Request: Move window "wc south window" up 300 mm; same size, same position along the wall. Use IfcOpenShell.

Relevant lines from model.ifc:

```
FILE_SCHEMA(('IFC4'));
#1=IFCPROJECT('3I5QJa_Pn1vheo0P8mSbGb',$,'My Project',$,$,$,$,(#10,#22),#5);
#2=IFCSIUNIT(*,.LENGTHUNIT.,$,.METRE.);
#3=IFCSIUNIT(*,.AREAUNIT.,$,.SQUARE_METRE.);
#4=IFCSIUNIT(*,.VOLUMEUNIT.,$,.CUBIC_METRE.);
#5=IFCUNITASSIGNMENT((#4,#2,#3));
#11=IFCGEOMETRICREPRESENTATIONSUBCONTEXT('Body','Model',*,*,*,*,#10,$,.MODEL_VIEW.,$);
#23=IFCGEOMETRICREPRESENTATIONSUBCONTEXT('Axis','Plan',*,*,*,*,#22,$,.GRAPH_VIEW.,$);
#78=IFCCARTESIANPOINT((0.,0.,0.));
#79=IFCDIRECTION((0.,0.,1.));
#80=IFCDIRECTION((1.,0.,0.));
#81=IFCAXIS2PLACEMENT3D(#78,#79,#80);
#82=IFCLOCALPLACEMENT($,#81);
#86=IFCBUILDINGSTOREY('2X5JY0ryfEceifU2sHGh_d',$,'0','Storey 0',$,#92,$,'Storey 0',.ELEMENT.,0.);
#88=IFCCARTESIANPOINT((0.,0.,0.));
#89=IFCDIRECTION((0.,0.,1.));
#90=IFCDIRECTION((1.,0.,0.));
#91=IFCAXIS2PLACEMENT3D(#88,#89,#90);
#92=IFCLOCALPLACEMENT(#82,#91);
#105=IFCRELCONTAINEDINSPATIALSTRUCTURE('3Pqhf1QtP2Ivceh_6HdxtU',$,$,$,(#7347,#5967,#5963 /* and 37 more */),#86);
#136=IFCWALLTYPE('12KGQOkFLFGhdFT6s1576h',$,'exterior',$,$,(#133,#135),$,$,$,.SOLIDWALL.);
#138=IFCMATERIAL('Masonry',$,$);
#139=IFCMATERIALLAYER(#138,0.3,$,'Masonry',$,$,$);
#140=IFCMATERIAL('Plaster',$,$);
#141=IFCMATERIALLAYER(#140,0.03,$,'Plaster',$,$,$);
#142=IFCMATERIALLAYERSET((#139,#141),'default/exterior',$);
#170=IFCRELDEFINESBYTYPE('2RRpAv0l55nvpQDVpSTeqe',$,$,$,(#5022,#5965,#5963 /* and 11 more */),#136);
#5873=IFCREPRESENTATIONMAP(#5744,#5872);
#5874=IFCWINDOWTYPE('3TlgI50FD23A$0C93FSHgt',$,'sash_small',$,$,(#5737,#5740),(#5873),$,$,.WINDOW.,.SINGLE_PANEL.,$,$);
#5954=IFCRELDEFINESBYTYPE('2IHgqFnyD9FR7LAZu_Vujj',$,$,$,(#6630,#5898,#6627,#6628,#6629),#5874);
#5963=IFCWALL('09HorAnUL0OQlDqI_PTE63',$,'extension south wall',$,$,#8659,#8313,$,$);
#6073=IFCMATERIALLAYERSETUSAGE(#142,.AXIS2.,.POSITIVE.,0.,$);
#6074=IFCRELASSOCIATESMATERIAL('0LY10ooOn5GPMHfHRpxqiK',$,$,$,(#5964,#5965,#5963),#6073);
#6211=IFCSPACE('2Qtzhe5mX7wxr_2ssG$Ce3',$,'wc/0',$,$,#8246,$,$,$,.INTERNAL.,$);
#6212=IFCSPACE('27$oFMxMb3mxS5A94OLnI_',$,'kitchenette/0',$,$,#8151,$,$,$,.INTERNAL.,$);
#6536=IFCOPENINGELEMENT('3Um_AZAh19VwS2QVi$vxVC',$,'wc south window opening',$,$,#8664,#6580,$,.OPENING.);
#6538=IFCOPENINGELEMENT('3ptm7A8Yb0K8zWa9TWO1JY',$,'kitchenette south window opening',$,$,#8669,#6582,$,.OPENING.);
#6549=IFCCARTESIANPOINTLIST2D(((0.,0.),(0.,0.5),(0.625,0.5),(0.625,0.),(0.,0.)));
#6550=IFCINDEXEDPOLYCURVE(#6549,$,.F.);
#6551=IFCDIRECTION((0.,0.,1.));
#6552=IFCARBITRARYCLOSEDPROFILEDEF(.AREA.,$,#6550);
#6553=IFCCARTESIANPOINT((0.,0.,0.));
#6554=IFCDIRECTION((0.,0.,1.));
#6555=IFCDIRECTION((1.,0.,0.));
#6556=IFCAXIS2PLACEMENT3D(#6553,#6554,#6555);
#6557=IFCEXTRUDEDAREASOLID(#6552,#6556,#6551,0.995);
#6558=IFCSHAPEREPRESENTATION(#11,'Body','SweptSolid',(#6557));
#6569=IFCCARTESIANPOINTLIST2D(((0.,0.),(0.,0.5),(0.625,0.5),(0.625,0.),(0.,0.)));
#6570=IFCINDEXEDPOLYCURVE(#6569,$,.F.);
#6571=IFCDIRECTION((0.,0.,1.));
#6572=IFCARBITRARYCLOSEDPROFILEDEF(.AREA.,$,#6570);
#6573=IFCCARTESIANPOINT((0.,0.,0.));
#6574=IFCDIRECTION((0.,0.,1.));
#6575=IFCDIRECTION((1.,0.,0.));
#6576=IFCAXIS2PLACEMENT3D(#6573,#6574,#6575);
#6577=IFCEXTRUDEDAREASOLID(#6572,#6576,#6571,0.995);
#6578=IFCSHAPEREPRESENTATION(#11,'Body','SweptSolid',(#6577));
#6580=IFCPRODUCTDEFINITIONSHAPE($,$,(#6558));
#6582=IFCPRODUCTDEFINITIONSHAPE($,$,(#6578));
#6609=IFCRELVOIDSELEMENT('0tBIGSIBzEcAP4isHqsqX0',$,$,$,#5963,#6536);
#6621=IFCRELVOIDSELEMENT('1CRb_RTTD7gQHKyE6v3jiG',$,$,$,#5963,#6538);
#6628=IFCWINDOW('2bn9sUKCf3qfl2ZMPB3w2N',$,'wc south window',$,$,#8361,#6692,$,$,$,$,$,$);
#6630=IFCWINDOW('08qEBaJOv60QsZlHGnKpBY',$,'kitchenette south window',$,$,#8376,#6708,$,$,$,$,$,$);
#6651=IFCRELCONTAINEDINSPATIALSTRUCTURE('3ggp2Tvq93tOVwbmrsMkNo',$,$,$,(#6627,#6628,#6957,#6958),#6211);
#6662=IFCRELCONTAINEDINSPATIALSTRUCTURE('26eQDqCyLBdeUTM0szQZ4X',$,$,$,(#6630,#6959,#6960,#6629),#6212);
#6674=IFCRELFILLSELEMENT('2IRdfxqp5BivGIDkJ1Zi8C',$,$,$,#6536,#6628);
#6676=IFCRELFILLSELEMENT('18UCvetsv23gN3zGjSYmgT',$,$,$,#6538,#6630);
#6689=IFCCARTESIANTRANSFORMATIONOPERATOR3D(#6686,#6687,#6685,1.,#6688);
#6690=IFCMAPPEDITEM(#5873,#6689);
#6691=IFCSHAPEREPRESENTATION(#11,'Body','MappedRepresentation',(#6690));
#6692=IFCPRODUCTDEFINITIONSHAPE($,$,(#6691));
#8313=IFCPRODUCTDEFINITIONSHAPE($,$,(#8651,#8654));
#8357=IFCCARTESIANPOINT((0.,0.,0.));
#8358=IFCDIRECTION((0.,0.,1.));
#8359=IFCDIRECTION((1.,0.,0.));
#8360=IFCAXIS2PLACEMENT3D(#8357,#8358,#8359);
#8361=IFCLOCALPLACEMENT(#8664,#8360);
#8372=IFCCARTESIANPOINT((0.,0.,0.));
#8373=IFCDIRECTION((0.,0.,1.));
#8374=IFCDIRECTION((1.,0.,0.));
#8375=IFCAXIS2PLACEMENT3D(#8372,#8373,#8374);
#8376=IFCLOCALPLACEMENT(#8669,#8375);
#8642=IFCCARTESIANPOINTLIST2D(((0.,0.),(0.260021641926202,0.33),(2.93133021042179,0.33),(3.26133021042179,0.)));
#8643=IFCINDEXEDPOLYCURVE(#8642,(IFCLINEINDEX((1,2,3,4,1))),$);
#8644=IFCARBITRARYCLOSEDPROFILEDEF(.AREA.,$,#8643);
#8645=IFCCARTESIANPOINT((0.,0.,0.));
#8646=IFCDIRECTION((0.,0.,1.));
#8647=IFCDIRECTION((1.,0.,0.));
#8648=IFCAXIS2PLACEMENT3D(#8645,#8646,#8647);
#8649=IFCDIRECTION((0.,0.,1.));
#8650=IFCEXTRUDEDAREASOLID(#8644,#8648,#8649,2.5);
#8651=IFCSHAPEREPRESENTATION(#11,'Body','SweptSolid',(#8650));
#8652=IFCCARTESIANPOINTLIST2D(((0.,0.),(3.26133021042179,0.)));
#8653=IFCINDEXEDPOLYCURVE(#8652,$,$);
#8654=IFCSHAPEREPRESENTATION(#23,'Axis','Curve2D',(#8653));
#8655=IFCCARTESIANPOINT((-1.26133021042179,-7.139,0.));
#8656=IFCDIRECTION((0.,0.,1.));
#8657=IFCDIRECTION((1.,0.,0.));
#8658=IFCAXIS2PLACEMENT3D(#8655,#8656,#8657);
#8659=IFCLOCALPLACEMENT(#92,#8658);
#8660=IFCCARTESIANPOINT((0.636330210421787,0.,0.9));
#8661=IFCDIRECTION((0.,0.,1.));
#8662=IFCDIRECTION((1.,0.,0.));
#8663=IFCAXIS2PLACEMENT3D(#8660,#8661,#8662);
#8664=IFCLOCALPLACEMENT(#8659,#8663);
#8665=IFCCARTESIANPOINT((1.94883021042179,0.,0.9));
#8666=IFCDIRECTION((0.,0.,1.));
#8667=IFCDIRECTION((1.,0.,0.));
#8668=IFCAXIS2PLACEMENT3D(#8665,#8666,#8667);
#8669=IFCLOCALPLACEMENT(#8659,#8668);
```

```python
import numpy as np
import ifcopenshell
import ifcopenshell.api.geometry
import ifcopenshell.util.placement
import ifcopenshell.util.unit

model = ifcopenshell.open("model.ifc")
unit_scale = ifcopenshell.util.unit.calculate_unit_scale(model)

window = model.by_id(6628)
opening = window.FillsVoids[0].RelatingOpeningElement
dz = 0.3

shift = np.array([0.0, 0.0, dz])
# The window is placed relative to its opening, so it follows when the opening moves.
matrix = ifcopenshell.util.placement.get_local_placement(opening.ObjectPlacement)
matrix[:3, 3] += shift
ifcopenshell.api.geometry.edit_object_placement(
    model, product=opening, matrix=matrix, is_si=False, should_transform_children=True
)

print(f"moved by {dz * unit_scale:+.3f} m")

model.write("model_updated.ifc")
```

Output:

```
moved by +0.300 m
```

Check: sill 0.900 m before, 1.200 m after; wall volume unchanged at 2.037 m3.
